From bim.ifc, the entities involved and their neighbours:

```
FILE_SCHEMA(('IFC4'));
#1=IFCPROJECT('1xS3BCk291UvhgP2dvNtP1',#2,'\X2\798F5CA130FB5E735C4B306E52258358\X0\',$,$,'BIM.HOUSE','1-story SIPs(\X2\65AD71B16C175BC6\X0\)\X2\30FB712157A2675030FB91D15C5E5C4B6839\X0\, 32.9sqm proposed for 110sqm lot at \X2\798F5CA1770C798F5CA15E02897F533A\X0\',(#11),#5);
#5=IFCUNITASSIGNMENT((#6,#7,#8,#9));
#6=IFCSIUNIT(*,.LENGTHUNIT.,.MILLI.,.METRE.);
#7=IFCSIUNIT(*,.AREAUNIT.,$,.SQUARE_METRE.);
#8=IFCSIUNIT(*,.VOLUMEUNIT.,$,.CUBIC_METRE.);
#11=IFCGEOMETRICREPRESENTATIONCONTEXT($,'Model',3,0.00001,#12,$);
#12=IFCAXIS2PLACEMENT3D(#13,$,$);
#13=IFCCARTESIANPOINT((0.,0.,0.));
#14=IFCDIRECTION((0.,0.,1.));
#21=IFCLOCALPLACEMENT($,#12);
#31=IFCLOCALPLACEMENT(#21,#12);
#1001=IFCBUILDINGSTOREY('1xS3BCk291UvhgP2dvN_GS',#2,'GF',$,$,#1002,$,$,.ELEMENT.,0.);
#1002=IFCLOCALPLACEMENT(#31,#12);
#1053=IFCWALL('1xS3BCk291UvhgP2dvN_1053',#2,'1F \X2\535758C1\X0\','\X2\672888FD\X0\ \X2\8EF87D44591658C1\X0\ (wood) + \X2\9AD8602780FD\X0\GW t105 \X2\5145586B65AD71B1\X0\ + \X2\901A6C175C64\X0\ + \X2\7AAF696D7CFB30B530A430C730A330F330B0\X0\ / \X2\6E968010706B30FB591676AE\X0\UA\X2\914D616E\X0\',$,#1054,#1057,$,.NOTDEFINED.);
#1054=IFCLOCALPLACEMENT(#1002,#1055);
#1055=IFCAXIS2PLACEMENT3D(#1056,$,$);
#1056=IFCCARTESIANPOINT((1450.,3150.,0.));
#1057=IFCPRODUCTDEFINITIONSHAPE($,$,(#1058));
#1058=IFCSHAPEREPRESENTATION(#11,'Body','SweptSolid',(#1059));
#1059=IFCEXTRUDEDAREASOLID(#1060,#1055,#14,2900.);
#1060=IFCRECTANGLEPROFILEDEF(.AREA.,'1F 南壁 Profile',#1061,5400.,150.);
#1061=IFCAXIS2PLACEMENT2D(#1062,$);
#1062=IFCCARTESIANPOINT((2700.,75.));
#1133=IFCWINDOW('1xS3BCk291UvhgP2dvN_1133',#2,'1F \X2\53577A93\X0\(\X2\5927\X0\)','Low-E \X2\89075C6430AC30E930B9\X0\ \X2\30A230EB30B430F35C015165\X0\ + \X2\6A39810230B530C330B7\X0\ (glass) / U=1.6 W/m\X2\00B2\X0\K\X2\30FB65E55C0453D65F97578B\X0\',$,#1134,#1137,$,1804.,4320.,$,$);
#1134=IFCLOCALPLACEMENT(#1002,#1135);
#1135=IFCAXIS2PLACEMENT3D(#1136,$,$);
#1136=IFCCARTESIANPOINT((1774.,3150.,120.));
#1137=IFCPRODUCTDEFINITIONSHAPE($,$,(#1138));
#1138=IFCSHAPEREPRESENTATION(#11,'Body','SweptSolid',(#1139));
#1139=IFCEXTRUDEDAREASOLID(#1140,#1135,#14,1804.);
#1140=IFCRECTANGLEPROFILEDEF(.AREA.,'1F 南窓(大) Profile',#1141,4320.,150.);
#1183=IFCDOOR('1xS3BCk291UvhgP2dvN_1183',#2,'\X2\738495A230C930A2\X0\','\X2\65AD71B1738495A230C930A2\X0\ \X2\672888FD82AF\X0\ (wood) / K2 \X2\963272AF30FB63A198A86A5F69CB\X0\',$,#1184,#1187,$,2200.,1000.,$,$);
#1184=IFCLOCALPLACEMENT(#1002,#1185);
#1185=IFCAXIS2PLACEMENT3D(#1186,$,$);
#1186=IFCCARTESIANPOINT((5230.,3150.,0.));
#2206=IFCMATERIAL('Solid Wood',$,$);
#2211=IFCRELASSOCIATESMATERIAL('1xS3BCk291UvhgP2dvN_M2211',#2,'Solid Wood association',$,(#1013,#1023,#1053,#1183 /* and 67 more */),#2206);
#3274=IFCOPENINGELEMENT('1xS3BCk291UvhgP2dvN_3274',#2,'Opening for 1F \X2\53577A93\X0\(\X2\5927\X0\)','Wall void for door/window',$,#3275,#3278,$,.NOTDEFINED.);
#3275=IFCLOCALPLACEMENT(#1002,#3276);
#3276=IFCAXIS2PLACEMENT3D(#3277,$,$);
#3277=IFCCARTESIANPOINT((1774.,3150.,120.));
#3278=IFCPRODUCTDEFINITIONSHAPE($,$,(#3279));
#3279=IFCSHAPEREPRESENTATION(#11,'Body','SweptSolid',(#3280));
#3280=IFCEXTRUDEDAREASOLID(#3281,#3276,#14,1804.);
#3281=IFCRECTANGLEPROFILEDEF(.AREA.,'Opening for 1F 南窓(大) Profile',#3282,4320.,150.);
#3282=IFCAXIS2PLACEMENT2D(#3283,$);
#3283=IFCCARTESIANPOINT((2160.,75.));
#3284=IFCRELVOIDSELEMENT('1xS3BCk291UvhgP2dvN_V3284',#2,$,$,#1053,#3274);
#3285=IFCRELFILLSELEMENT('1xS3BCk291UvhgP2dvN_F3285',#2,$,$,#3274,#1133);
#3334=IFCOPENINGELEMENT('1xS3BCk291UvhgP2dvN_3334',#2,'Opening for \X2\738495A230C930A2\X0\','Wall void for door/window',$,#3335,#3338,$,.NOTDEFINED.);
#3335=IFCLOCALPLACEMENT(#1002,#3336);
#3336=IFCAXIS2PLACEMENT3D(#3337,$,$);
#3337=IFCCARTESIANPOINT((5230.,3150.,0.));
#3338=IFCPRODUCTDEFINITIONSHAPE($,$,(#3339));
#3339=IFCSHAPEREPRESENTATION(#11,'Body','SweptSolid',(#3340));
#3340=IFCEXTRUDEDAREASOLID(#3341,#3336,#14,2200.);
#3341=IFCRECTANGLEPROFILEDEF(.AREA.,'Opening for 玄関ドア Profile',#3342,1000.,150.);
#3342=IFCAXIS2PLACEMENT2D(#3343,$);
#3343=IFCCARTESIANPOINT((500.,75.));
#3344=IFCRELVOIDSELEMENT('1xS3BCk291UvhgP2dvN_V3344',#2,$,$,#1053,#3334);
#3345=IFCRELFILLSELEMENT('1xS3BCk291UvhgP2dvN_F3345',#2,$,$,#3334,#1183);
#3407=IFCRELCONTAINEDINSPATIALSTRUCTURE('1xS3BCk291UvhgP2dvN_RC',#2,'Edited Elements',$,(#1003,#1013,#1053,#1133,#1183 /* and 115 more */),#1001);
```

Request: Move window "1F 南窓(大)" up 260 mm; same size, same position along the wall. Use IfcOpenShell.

```python
import numpy as np
import ifcopenshell
import ifcopenshell.api.geometry
import ifcopenshell.util.placement
import ifcopenshell.util.unit

model = ifcopenshell.open("bim.ifc")
unit_scale = ifcopenshell.util.unit.calculate_unit_scale(model)

window = model.by_guid("1xS3BCk291UvhgP2dvN_1133")
opening = window.FillsVoids[0].RelatingOpeningElement
dz = 260.0

shift = np.array([0.0, 0.0, dz])
# The window is not placed relative to its opening, so move both.
for product in (opening, window):
    matrix = ifcopenshell.util.placement.get_local_placement(product.ObjectPlacement)
    matrix[:3, 3] += shift
    ifcopenshell.api.geometry.edit_object_placement(model, product=product, matrix=matrix, is_si=False)

print(f"moved by {dz * unit_scale:+.3f} m")

model.write("bim_rev.ifc")
```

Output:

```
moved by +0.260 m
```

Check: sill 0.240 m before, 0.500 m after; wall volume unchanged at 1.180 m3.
